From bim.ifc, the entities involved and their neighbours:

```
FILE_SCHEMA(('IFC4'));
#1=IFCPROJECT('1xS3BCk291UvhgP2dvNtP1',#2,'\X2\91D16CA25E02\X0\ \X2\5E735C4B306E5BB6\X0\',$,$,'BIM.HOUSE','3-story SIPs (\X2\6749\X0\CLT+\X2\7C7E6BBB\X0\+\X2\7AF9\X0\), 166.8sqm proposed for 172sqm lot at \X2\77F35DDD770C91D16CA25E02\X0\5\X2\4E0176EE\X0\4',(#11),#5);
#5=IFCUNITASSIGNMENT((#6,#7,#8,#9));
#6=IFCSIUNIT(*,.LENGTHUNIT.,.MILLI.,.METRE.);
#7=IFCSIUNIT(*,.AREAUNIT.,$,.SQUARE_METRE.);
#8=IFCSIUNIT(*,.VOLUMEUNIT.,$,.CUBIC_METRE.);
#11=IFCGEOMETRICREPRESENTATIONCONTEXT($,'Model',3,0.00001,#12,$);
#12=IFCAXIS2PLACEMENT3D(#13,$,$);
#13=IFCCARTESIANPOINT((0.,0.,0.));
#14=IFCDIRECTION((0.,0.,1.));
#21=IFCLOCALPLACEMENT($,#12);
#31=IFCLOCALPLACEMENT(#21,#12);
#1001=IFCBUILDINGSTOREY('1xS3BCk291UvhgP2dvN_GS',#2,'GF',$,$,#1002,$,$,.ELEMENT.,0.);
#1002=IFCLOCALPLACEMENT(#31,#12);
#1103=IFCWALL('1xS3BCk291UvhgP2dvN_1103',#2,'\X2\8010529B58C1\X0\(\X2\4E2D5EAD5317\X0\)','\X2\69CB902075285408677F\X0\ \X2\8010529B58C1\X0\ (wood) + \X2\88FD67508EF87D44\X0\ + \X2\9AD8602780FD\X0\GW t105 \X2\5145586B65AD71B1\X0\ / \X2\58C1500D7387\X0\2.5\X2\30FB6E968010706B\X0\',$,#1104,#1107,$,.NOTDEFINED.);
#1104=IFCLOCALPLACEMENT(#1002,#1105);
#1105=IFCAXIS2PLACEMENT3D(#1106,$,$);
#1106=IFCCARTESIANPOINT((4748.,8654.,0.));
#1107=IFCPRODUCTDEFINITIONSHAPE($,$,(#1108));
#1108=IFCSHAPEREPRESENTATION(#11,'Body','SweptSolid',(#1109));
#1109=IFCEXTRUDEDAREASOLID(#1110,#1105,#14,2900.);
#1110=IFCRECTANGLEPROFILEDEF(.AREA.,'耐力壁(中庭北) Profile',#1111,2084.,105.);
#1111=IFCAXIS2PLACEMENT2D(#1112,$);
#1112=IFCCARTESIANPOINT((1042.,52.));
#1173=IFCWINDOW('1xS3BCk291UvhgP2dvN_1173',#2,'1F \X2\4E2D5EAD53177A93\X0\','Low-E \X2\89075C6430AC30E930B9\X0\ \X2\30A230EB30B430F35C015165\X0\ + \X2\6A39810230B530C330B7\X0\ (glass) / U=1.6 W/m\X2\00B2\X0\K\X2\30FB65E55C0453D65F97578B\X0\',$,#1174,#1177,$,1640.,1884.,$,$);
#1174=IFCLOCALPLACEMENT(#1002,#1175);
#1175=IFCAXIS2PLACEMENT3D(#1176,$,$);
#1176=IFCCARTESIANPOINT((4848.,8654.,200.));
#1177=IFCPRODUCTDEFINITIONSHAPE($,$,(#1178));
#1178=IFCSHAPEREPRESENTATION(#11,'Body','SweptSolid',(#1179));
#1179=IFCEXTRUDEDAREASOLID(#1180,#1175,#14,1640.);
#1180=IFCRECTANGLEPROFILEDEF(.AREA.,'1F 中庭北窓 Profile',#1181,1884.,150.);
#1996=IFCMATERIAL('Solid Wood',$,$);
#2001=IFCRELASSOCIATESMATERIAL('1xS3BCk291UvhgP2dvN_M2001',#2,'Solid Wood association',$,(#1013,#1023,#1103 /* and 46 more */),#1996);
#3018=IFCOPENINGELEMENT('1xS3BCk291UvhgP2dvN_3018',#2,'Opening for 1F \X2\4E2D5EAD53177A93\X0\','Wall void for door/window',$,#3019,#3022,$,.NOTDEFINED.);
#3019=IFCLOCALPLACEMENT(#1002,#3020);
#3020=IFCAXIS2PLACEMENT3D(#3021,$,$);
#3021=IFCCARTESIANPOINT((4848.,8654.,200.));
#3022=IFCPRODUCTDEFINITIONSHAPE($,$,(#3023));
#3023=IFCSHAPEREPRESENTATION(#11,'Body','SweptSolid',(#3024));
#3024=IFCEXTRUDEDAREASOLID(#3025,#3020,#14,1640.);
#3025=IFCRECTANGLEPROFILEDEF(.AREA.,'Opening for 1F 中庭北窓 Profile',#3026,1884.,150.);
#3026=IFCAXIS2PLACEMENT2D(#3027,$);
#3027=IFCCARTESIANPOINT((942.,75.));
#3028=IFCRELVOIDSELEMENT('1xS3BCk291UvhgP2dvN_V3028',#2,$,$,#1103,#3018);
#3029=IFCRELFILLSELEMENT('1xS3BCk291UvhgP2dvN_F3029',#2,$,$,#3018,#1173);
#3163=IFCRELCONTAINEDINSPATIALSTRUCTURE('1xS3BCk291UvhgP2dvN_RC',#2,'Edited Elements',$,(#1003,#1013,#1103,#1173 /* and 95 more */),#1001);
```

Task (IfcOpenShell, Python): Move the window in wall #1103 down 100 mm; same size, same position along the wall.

```python
import numpy as np
import ifcopenshell
import ifcopenshell.api.geometry
import ifcopenshell.util.placement
import ifcopenshell.util.unit

model = ifcopenshell.open("bim.ifc")
unit_scale = ifcopenshell.util.unit.calculate_unit_scale(model)

window = model.by_guid("1xS3BCk291UvhgP2dvN_1173")
opening = window.FillsVoids[0].RelatingOpeningElement
dz = -0.1 / unit_scale

shift = np.array([0.0, 0.0, dz])
# The window is not placed relative to its opening, so move both.
for product in (opening, window):
    matrix = ifcopenshell.util.placement.get_local_placement(product.ObjectPlacement)
    matrix[:3, 3] += shift
    ifcopenshell.api.geometry.edit_object_placement(model, product=product, matrix=matrix, is_si=False)

print(f"moved by {dz * unit_scale:+.3f} m")

model.write("bim_edited.ifc")
```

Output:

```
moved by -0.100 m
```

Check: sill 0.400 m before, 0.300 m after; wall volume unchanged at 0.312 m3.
